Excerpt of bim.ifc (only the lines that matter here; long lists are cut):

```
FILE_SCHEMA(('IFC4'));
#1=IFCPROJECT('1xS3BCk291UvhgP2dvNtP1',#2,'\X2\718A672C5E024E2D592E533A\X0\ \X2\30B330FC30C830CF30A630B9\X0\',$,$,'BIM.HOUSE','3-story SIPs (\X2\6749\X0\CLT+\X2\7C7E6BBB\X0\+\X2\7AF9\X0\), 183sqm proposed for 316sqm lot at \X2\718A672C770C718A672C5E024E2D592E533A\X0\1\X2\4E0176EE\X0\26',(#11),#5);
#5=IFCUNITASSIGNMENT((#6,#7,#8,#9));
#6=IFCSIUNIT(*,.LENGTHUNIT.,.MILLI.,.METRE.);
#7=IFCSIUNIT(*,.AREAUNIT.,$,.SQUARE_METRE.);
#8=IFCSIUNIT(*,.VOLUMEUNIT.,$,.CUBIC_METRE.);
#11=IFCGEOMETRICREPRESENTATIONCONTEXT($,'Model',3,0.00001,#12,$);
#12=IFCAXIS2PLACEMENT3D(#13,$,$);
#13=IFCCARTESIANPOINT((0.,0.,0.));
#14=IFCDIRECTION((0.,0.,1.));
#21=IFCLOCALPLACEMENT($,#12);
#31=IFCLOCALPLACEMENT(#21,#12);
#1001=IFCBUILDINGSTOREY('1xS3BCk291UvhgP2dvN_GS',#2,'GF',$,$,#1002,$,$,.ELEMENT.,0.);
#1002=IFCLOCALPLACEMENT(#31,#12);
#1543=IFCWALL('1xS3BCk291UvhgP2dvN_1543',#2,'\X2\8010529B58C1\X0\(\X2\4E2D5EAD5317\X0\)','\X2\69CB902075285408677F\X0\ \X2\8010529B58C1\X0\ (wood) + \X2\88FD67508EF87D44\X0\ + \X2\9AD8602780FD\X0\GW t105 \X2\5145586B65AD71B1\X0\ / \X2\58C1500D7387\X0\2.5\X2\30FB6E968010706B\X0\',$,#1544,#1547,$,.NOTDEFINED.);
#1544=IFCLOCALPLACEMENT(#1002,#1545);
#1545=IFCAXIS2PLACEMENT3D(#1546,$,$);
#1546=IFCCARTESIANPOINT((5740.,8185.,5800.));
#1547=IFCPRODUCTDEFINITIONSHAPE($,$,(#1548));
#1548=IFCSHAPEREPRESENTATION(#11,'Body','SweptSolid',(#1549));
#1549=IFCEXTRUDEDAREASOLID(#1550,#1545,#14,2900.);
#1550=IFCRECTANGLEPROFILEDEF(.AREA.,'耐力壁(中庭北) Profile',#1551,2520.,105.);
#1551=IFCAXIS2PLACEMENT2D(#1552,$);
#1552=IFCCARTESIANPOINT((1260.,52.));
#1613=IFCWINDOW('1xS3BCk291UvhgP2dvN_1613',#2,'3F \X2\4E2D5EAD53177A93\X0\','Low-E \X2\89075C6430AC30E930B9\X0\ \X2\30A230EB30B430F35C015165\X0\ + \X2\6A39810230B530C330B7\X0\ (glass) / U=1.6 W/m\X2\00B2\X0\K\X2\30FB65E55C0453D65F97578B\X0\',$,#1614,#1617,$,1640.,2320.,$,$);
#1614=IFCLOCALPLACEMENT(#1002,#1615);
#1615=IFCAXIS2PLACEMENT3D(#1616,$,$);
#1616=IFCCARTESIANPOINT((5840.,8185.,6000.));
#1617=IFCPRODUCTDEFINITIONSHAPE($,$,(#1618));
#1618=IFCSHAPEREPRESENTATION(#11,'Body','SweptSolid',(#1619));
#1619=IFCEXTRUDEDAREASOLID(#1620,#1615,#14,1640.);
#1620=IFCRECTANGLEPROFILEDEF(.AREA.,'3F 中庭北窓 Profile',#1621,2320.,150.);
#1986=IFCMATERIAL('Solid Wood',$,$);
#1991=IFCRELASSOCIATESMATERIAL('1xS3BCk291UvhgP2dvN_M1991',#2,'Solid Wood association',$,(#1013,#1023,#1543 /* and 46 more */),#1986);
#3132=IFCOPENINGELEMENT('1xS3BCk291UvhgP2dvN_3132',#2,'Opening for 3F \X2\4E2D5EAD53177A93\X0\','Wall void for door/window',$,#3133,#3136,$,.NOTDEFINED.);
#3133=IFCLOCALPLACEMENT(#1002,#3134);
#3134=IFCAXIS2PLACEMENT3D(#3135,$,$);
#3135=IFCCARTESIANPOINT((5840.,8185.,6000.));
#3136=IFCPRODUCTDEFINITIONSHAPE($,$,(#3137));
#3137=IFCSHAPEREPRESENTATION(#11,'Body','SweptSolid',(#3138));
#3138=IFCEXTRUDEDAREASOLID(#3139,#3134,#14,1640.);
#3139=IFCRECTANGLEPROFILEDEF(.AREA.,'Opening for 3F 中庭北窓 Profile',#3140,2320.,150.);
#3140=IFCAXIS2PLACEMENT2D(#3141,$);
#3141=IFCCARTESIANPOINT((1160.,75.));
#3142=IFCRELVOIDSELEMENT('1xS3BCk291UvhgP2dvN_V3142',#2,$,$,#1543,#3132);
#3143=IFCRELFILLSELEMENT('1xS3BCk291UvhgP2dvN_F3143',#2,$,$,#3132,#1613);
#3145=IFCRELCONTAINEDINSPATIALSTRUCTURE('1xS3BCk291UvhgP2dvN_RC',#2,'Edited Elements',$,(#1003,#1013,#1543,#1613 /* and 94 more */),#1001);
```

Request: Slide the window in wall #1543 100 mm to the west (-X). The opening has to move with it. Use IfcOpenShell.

```python
import ifcopenshell
import ifcopenshell.api.geometry
import ifcopenshell.util.placement
import ifcopenshell.util.unit

model = ifcopenshell.open("bim.ifc")
unit_scale = ifcopenshell.util.unit.calculate_unit_scale(model)

window = model.by_id(1613)
opening = window.FillsVoids[0].RelatingOpeningElement
wall = opening.VoidsElements[0].RelatingBuildingElement

wall_matrix = ifcopenshell.util.placement.get_local_placement(wall.ObjectPlacement)
shift = wall_matrix[:3, 0] * -0.1 / unit_scale
before = ifcopenshell.util.placement.get_local_placement(window.ObjectPlacement)[:3, 3].copy()

# The window is not placed relative to its opening, so move both.
for product in (opening, window):
    matrix = ifcopenshell.util.placement.get_local_placement(product.ObjectPlacement)
    matrix[:3, 3] += shift
    ifcopenshell.api.geometry.edit_object_placement(model, product=product, matrix=matrix, is_si=False)

after = ifcopenshell.util.placement.get_local_placement(window.ObjectPlacement)[:3, 3]
print("window moved by", (after - before).round(3) + 0.0)

model.write("bim_edited.ifc")
```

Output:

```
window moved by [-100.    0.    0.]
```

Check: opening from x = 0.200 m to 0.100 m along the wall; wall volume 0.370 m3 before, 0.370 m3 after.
